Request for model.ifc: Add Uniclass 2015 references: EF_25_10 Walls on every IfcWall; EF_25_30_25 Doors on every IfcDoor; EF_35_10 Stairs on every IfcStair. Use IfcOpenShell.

First a look at what the model holds.

```python
import ifcopenshell

model = ifcopenshell.open("model.ifc")
print(model.schema)
print("classifications:", [c.Name for c in model.by_type("IfcClassification")])
for ifc_class in ("IfcDoor", "IfcRoof", "IfcStair", "IfcWall", "IfcWindow"):
    print(ifc_class, len(model.by_type(ifc_class)))
```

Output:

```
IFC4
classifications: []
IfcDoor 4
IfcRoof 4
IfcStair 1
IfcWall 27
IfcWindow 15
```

```python
import ifcopenshell
import ifcopenshell.api.classification

model = ifcopenshell.open("model.ifc")

system = ifcopenshell.api.classification.add_classification(model, classification="Uniclass 2015")

codes = {
    "IfcWall": ("EF_25_10", "Walls"),
    "IfcDoor": ("EF_25_30_25", "Doors"),
    "IfcStair": ("EF_35_10", "Stairs"),
}
for ifc_class, (code, name) in codes.items():
    products = model.by_type(ifc_class)
    ifcopenshell.api.classification.add_reference(
        model, products=products, classification=system, identification=code, name=name
    )
    print(code, len(products))

model.write("model_edited.ifc")
```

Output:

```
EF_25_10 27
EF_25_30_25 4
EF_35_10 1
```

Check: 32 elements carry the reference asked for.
